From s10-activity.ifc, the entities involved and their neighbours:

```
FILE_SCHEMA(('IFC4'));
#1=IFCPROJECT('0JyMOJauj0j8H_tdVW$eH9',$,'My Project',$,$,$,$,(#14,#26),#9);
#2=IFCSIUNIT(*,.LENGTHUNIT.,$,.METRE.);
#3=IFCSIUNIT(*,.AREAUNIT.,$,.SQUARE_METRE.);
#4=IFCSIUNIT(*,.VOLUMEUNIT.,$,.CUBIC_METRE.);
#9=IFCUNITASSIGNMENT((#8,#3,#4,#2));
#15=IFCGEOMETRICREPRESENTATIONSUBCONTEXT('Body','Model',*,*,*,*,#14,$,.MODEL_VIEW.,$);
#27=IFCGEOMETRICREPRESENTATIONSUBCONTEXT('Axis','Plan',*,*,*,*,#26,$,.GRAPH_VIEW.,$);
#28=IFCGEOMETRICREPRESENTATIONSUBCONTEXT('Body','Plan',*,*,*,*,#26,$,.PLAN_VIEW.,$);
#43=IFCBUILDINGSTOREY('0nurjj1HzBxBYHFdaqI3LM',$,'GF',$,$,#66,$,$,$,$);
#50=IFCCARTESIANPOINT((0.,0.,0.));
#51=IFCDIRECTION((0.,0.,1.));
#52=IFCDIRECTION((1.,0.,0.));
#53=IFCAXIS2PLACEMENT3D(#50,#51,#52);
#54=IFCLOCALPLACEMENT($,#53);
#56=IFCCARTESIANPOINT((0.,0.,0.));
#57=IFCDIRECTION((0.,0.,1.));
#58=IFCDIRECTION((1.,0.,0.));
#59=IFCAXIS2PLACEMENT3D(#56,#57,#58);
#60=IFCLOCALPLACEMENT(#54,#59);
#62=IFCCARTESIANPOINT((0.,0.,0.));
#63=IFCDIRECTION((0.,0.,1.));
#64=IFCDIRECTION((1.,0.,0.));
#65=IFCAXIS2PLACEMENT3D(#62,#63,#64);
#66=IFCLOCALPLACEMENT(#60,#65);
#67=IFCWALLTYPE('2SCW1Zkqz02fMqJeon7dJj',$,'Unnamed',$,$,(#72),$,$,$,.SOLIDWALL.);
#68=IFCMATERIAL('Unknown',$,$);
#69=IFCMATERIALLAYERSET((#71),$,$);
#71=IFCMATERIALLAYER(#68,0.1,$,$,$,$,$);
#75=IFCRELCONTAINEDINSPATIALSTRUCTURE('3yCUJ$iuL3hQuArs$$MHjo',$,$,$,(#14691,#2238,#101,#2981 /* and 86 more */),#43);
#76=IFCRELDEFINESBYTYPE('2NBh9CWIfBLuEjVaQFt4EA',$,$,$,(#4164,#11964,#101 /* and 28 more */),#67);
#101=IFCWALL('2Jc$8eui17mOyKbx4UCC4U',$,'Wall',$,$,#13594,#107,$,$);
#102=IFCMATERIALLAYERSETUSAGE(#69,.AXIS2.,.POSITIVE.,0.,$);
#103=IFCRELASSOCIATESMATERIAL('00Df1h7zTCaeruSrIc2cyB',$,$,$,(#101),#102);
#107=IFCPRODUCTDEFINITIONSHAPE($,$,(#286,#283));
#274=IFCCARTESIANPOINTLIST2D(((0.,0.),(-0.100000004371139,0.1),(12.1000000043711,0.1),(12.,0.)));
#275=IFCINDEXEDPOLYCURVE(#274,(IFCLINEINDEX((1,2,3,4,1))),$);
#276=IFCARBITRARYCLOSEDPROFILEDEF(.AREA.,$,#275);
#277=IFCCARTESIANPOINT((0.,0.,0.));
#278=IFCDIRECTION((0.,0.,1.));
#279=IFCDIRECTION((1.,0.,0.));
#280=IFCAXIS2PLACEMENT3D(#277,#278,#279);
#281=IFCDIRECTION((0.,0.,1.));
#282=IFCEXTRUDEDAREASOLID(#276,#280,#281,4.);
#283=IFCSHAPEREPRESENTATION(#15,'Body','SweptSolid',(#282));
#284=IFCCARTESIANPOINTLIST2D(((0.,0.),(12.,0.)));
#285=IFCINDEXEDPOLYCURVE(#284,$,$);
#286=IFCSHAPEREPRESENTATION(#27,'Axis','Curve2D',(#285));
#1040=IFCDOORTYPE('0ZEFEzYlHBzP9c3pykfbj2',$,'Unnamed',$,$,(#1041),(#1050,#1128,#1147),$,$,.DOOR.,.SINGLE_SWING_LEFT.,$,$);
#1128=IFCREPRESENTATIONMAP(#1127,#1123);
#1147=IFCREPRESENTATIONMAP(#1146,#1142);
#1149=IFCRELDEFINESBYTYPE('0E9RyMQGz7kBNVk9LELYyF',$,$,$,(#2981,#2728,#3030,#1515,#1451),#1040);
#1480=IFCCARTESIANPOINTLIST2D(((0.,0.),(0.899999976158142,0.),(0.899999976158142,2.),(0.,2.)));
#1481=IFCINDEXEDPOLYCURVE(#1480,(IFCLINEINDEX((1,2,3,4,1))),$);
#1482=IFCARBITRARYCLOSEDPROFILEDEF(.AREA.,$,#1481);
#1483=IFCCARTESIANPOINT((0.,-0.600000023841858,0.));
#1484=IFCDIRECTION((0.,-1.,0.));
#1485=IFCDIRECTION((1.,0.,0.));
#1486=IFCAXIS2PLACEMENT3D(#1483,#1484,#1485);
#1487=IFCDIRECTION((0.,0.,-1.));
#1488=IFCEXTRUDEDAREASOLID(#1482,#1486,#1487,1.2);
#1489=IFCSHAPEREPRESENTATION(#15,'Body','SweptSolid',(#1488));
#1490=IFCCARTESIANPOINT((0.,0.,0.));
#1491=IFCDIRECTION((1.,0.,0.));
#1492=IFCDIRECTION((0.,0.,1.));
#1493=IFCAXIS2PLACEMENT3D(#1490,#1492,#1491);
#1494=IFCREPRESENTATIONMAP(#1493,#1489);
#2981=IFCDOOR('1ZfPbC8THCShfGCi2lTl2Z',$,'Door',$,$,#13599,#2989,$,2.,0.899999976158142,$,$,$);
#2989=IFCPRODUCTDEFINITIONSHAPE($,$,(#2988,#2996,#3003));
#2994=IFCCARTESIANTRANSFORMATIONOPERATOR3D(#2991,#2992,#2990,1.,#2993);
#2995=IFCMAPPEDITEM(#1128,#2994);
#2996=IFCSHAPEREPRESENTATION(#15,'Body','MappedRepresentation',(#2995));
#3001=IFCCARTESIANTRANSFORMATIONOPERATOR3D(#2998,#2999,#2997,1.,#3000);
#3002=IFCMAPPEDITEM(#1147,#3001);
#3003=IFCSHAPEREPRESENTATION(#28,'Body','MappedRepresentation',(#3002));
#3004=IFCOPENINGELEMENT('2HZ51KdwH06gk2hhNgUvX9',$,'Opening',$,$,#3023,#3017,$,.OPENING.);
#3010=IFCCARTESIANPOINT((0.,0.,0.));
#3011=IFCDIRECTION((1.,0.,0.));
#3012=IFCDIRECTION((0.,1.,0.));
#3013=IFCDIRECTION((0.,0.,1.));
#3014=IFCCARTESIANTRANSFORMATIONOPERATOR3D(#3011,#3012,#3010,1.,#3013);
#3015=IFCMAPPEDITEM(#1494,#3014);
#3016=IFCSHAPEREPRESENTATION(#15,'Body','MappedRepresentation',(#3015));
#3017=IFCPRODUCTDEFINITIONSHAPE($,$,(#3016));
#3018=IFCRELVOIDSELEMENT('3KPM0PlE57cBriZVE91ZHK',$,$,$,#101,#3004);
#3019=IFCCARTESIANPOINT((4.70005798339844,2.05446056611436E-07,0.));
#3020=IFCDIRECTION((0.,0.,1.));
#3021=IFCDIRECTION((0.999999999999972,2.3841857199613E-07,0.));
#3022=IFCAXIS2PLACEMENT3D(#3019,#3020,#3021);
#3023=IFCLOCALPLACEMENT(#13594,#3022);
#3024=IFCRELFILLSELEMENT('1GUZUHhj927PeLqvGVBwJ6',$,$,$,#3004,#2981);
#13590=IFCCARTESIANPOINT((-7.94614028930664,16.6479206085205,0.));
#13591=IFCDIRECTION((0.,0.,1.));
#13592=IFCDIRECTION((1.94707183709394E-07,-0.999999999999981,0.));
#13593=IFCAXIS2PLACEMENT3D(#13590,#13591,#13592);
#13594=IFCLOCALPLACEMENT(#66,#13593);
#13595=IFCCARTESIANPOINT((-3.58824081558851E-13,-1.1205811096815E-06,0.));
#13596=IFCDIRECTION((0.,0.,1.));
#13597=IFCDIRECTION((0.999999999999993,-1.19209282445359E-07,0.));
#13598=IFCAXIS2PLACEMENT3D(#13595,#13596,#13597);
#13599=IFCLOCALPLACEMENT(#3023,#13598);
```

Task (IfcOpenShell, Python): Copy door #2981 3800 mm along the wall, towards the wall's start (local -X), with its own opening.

```python
import ifcopenshell
import ifcopenshell.api.feature
import ifcopenshell.api.geometry
import ifcopenshell.api.root
import ifcopenshell.geom
import ifcopenshell.util.element
import ifcopenshell.util.placement
import ifcopenshell.util.shape

model = ifcopenshell.open("s10-activity.ifc")
settings = ifcopenshell.geom.settings()


def volume(element):
    """Net volume in cubic metres, openings subtracted."""
    shape = ifcopenshell.geom.create_shape(settings, element)
    return ifcopenshell.util.shape.get_volume(shape.geometry)


door = model.by_guid("1ZfPbC8THCShfGCi2lTl2Z")
opening = door.FillsVoids[0].RelatingOpeningElement
wall = opening.VoidsElements[0].RelatingBuildingElement
before = volume(wall)
shift = ifcopenshell.util.placement.get_local_placement(wall.ObjectPlacement)[:3, 0] * -3.8

# copy_class copies the void relationship, type, container and properties, but no geometry.
new_opening = ifcopenshell.api.root.copy_class(model, product=opening)
new_opening.Representation = ifcopenshell.util.element.copy_deep(
    model, opening.Representation, exclude=["IfcGeometricRepresentationContext", "IfcRepresentationMap"]
)
new_door = ifcopenshell.api.root.copy_class(model, product=door)
new_door.Representation = ifcopenshell.util.element.copy_deep(
    model, door.Representation, exclude=["IfcGeometricRepresentationContext", "IfcRepresentationMap"]
)
ifcopenshell.api.feature.add_filling(model, opening=new_opening, element=new_door)

for old, new in ((opening, new_opening), (door, new_door)):
    matrix = ifcopenshell.util.placement.get_local_placement(old.ObjectPlacement)
    matrix[:3, 3] += shift
    ifcopenshell.api.geometry.edit_object_placement(model, product=new, matrix=matrix, is_si=False)

after = volume(wall)

print(f"wall volume {before:.3f} -> {after:.3f} m3")

model.write("s10-activity_v2.ifc")
```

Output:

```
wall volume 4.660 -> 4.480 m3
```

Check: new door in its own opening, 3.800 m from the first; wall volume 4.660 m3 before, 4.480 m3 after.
